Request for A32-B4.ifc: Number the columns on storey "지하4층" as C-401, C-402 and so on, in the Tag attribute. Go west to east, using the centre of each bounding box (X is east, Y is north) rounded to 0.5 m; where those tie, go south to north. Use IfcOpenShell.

First a look at what the model holds.

```python
import ifcopenshell
import ifcopenshell.util.element
import ifcopenshell.util.placement

model = ifcopenshell.open("A32-B4.ifc")
print(model.schema)
storey = next(s for s in model.by_type("IfcBuildingStorey") if s.Name == "지하4층")
columns = [e for e in ifcopenshell.util.element.get_decomposition(storey) if e.is_a("IfcColumn")]
for e in sorted(columns, key=lambda e: e.id()):
    origin = ifcopenshell.util.placement.get_local_placement(e.ObjectPlacement)[:3, 3]
    print(e.id(), e.Tag, e.Name, origin.round(2) + 0.0, sep=" | ")
```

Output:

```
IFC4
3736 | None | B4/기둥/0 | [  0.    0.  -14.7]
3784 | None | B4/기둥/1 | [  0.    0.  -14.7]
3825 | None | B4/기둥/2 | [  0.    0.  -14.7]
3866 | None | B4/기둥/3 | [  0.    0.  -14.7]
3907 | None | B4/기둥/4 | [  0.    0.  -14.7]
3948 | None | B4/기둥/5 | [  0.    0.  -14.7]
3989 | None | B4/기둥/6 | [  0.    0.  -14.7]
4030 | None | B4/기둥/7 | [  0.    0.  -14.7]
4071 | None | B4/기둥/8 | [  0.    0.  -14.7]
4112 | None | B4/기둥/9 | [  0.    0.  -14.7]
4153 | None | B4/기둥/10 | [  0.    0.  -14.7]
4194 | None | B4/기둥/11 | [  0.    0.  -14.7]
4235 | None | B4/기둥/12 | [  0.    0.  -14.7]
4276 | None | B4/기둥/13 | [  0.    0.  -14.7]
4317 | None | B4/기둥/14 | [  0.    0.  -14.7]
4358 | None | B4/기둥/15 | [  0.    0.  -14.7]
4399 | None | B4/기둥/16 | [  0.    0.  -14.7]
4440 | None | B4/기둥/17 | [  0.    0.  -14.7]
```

```python
import ifcopenshell
import ifcopenshell.geom
import ifcopenshell.util.element
import ifcopenshell.util.shape

model = ifcopenshell.open("A32-B4.ifc")
settings = ifcopenshell.geom.settings()
settings.set("use-world-coords", True)


def centre(element):
    shape = ifcopenshell.geom.create_shape(settings, element)
    return ifcopenshell.util.shape.get_bbox_centroid(shape.geometry)


storey = next(s for s in model.by_type("IfcBuildingStorey") if s.Name == "지하4층")
columns = [e for e in ifcopenshell.util.element.get_decomposition(storey) if e.is_a("IfcColumn")]

# Insertion points can sit at a corner or the storey origin, so sort by the geometry (in metres).
centres = {e: centre(e) for e in columns}
columns.sort(key=lambda e: (round(centres[e][0] / 0.5), centres[e][1]))

for i, e in enumerate(columns, start=1):
    number = f"C-4{i:02d}"
    e.Tag = number
    print(e.id(), number)

model.write("A32-B4_v2.ifc")
```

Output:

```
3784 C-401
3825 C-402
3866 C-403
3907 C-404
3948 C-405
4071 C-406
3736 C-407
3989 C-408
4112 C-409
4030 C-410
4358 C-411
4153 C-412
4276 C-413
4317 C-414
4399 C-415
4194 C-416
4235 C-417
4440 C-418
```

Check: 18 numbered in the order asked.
